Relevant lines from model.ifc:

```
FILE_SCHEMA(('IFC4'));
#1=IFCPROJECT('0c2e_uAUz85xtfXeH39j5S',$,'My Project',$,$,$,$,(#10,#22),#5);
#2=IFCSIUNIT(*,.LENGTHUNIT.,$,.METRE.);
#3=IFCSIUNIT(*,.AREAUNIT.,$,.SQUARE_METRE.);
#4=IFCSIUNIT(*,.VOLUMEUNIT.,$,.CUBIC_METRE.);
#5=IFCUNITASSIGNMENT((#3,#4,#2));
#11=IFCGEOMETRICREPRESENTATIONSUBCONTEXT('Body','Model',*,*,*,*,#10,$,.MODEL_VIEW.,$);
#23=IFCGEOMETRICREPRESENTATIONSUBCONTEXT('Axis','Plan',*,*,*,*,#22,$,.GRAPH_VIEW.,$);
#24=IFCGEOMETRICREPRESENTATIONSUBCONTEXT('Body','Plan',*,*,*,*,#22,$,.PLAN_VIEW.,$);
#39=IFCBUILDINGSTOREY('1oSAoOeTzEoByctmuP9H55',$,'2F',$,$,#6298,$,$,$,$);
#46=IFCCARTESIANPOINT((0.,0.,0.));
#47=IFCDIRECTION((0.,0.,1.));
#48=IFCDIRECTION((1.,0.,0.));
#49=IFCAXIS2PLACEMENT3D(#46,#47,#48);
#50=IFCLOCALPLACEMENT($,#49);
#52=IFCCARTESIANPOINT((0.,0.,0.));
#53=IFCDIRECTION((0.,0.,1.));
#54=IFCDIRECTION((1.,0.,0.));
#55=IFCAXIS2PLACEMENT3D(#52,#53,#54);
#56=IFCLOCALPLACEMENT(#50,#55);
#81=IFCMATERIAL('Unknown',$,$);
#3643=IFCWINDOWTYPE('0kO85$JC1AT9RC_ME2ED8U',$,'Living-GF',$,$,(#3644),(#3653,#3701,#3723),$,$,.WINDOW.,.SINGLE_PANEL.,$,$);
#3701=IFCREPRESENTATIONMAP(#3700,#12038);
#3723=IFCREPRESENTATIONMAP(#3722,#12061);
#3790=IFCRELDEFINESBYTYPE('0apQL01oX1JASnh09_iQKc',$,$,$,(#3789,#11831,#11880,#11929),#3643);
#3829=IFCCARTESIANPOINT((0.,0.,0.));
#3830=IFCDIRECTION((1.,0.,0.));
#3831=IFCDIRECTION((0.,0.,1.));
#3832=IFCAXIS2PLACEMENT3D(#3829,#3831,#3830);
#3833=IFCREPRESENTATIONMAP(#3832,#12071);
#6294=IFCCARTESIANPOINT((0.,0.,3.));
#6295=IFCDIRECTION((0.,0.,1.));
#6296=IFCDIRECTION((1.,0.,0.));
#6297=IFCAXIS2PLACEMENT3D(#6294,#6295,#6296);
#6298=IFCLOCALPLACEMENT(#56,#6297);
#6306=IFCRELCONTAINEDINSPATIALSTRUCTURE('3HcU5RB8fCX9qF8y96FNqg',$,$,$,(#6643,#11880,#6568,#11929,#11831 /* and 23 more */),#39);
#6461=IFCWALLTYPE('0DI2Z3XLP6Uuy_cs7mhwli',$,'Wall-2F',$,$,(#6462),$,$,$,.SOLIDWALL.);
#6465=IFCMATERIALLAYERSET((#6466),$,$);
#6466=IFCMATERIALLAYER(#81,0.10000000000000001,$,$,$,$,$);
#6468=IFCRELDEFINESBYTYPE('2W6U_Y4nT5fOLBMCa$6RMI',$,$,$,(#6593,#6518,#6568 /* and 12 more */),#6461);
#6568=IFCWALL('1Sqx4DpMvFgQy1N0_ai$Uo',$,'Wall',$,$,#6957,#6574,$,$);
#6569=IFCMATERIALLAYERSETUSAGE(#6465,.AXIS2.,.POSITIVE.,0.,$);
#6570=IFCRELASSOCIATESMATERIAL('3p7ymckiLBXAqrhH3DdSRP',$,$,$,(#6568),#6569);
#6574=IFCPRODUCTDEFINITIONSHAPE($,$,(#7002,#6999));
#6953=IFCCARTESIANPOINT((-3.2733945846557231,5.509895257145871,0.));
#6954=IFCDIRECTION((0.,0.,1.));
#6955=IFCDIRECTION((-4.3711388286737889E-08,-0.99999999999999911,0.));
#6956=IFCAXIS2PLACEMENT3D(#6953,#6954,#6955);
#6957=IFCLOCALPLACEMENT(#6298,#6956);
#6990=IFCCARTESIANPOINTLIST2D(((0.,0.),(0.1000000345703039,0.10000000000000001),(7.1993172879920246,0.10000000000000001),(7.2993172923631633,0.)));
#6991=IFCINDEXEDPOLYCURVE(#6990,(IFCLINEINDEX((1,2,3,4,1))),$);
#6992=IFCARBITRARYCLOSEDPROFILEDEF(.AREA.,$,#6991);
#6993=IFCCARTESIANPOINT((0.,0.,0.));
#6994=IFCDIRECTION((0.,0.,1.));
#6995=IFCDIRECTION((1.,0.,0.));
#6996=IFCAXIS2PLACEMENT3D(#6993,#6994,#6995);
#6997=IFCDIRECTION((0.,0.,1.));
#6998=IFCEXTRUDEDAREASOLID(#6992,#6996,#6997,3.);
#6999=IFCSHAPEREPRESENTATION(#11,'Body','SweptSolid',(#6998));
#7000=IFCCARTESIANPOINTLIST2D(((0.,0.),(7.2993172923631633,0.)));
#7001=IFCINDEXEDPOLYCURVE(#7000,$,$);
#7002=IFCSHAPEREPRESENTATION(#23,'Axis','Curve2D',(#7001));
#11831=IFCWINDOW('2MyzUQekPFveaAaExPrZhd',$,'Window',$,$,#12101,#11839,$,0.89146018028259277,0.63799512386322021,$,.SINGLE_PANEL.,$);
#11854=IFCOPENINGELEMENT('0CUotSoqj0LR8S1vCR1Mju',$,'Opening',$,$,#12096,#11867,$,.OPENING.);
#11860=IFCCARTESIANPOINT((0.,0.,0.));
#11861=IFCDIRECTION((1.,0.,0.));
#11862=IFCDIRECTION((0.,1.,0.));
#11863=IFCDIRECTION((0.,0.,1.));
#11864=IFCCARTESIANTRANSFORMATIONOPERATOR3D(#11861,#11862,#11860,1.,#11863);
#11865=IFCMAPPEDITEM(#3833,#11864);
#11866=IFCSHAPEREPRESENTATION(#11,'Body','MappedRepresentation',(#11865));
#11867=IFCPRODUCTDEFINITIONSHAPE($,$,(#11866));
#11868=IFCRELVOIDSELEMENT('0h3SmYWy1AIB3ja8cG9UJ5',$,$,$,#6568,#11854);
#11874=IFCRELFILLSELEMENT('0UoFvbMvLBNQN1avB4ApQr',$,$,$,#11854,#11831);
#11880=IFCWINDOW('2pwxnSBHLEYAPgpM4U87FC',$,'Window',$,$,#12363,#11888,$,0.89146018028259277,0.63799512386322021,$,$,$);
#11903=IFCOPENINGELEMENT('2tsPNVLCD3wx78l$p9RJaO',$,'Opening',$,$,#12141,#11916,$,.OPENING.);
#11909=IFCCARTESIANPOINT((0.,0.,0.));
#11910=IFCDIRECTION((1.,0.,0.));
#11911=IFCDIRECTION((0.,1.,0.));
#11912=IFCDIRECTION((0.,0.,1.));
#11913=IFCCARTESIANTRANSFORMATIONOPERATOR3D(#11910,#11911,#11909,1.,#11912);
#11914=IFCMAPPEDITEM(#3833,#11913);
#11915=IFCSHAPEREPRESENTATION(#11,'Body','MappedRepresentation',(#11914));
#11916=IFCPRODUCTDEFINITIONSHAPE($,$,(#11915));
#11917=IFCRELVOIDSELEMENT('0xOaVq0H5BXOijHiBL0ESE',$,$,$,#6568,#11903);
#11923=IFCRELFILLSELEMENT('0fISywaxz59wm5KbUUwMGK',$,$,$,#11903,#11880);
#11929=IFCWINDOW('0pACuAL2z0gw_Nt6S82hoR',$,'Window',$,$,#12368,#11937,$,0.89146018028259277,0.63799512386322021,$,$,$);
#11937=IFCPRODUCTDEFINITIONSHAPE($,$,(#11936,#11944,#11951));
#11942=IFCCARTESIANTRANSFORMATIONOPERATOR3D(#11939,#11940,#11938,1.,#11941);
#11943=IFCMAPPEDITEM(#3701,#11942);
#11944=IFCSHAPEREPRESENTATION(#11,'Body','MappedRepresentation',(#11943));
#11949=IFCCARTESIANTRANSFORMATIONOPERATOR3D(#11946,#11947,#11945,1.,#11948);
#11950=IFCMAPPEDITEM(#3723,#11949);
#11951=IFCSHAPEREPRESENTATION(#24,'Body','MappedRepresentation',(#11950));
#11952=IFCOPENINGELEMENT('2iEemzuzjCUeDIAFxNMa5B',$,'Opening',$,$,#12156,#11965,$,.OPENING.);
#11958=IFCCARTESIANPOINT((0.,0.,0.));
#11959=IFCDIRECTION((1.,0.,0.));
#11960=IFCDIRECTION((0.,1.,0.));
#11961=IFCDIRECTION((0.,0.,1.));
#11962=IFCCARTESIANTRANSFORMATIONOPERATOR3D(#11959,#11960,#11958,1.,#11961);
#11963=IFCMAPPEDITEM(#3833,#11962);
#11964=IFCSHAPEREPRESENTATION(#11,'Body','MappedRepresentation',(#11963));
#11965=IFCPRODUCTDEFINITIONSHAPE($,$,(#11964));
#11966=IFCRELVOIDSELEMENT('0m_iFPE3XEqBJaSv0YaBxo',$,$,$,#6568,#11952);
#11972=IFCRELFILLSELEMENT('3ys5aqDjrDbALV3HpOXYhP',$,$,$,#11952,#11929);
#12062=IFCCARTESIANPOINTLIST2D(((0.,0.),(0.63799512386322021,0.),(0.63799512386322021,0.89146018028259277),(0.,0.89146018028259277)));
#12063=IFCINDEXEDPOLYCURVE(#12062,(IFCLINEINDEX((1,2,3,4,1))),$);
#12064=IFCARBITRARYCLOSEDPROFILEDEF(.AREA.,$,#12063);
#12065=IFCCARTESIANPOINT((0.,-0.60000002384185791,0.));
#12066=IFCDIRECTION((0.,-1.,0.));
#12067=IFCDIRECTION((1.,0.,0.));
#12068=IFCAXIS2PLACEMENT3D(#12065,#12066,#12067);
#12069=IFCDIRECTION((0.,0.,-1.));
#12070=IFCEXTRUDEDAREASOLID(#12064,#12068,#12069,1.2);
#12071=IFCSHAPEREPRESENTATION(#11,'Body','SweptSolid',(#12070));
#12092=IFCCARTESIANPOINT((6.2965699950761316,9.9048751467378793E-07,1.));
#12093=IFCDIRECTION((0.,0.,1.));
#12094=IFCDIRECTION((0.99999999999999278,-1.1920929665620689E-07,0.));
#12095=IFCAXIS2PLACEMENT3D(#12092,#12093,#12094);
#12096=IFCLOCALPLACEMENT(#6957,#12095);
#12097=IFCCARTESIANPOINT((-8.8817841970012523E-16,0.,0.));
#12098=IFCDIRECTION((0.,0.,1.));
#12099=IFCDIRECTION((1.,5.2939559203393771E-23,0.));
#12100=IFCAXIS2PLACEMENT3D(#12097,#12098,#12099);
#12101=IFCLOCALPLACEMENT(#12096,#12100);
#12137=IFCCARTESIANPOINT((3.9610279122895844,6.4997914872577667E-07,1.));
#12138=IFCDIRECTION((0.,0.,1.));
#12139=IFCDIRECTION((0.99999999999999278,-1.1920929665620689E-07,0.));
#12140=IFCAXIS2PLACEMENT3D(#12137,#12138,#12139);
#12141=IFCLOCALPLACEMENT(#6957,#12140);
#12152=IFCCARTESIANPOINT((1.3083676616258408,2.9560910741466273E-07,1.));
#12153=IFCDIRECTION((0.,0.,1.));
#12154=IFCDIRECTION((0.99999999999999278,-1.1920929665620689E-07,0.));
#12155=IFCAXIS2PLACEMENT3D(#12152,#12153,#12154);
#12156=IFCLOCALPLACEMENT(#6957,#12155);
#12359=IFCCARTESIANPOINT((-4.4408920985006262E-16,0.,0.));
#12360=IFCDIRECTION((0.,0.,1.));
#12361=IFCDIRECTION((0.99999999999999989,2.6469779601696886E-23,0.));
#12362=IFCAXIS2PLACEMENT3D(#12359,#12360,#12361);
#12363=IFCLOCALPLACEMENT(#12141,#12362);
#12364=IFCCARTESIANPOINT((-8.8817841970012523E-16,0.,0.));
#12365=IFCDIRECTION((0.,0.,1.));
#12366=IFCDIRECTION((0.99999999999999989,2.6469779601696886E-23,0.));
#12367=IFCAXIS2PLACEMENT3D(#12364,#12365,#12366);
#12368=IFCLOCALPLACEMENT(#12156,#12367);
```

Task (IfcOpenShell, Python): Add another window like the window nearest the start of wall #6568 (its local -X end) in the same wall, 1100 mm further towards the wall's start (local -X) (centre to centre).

```python
import ifcopenshell
import ifcopenshell.api.feature
import ifcopenshell.api.geometry
import ifcopenshell.api.root
import ifcopenshell.geom
import ifcopenshell.util.element
import ifcopenshell.util.placement
import ifcopenshell.util.shape

model = ifcopenshell.open("model.ifc")
settings = ifcopenshell.geom.settings()


def volume(element):
    """Net volume in cubic metres, openings subtracted."""
    shape = ifcopenshell.geom.create_shape(settings, element)
    return ifcopenshell.util.shape.get_volume(shape.geometry)


window = model.by_guid("0pACuAL2z0gw_Nt6S82hoR")
opening = window.FillsVoids[0].RelatingOpeningElement
wall = opening.VoidsElements[0].RelatingBuildingElement
before = volume(wall)
shift = ifcopenshell.util.placement.get_local_placement(wall.ObjectPlacement)[:3, 0] * -1.1

# copy_class copies the void relationship, type, container and properties, but no geometry.
new_opening = ifcopenshell.api.root.copy_class(model, product=opening)
new_opening.Representation = ifcopenshell.util.element.copy_deep(
    model, opening.Representation, exclude=["IfcGeometricRepresentationContext", "IfcRepresentationMap"]
)
new_window = ifcopenshell.api.root.copy_class(model, product=window)
new_window.Representation = ifcopenshell.util.element.copy_deep(
    model, window.Representation, exclude=["IfcGeometricRepresentationContext", "IfcRepresentationMap"]
)
ifcopenshell.api.feature.add_filling(model, opening=new_opening, element=new_window)

for old, new in ((opening, new_opening), (window, new_window)):
    matrix = ifcopenshell.util.placement.get_local_placement(old.ObjectPlacement)
    matrix[:3, 3] += shift
    ifcopenshell.api.geometry.edit_object_placement(model, product=new, matrix=matrix, is_si=False)

after = volume(wall)

print(f"wall volume {before:.3f} -> {after:.3f} m3")

model.write("model_edited.ifc")
```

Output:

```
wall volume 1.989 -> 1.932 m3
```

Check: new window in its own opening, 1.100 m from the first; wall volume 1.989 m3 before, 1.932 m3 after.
